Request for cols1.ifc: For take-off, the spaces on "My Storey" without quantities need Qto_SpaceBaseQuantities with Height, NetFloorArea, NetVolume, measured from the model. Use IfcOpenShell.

First a look at what the model holds.

```python
import ifcopenshell
import ifcopenshell.util.element
import ifcopenshell.util.unit

model = ifcopenshell.open("cols1.ifc")
print(model.schema)
for unit_type in ("LENGTHUNIT", "AREAUNIT", "VOLUMEUNIT"):
    print(unit_type, ifcopenshell.util.unit.calculate_unit_scale(model, unit_type))
storey = next(s for s in model.by_type("IfcBuildingStorey") if s.Name == "My Storey")
spaces = [e for e in ifcopenshell.util.element.get_decomposition(storey) if e.is_a("IfcSpace")]
for e in sorted(spaces, key=lambda e: e.id()):
    print(e.id(), e.is_a(), e.Name, list(ifcopenshell.util.element.get_psets(e, qtos_only=True)), sep=" | ")
```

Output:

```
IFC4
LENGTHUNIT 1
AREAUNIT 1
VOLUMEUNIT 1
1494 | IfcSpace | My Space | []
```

```python
import ifcopenshell
import ifcopenshell.api.pset
import ifcopenshell.geom
import ifcopenshell.util.element
import ifcopenshell.util.shape
import ifcopenshell.util.unit

model = ifcopenshell.open("cols1.ifc")
unit_scale = ifcopenshell.util.unit.calculate_unit_scale(model)
area_scale = ifcopenshell.util.unit.calculate_unit_scale(model, "AREAUNIT")
volume_scale = ifcopenshell.util.unit.calculate_unit_scale(model, "VOLUMEUNIT")
settings = ifcopenshell.geom.settings()

storey = next(s for s in model.by_type("IfcBuildingStorey") if s.Name == "My Storey")
spaces = [e for e in ifcopenshell.util.element.get_decomposition(storey) if e.is_a("IfcSpace")]

for e in sorted(spaces, key=lambda e: e.id()):
    if ifcopenshell.util.element.get_psets(e, qtos_only=True, should_inherit=False):
        continue
    # Geometry comes back in metres, in the element's own axes.
    shape = ifcopenshell.geom.create_shape(settings, e)
    values = {
        "Height": ifcopenshell.util.shape.get_z(shape.geometry) / unit_scale,
        "NetFloorArea": ifcopenshell.util.shape.get_footprint_area(shape.geometry) / area_scale,
        "NetVolume": ifcopenshell.util.shape.get_volume(shape.geometry) / volume_scale,
    }
    qto = ifcopenshell.api.pset.add_qto(model, product=e, name="Qto_SpaceBaseQuantities")
    ifcopenshell.api.pset.edit_qto(model, qto=qto, properties=values)
    print(e.id(), {k: round(v, 3) for k, v in values.items()})

model.write("cols1_rev.ifc")
```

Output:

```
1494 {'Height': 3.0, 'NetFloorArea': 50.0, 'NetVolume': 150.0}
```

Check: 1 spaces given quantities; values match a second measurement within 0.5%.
